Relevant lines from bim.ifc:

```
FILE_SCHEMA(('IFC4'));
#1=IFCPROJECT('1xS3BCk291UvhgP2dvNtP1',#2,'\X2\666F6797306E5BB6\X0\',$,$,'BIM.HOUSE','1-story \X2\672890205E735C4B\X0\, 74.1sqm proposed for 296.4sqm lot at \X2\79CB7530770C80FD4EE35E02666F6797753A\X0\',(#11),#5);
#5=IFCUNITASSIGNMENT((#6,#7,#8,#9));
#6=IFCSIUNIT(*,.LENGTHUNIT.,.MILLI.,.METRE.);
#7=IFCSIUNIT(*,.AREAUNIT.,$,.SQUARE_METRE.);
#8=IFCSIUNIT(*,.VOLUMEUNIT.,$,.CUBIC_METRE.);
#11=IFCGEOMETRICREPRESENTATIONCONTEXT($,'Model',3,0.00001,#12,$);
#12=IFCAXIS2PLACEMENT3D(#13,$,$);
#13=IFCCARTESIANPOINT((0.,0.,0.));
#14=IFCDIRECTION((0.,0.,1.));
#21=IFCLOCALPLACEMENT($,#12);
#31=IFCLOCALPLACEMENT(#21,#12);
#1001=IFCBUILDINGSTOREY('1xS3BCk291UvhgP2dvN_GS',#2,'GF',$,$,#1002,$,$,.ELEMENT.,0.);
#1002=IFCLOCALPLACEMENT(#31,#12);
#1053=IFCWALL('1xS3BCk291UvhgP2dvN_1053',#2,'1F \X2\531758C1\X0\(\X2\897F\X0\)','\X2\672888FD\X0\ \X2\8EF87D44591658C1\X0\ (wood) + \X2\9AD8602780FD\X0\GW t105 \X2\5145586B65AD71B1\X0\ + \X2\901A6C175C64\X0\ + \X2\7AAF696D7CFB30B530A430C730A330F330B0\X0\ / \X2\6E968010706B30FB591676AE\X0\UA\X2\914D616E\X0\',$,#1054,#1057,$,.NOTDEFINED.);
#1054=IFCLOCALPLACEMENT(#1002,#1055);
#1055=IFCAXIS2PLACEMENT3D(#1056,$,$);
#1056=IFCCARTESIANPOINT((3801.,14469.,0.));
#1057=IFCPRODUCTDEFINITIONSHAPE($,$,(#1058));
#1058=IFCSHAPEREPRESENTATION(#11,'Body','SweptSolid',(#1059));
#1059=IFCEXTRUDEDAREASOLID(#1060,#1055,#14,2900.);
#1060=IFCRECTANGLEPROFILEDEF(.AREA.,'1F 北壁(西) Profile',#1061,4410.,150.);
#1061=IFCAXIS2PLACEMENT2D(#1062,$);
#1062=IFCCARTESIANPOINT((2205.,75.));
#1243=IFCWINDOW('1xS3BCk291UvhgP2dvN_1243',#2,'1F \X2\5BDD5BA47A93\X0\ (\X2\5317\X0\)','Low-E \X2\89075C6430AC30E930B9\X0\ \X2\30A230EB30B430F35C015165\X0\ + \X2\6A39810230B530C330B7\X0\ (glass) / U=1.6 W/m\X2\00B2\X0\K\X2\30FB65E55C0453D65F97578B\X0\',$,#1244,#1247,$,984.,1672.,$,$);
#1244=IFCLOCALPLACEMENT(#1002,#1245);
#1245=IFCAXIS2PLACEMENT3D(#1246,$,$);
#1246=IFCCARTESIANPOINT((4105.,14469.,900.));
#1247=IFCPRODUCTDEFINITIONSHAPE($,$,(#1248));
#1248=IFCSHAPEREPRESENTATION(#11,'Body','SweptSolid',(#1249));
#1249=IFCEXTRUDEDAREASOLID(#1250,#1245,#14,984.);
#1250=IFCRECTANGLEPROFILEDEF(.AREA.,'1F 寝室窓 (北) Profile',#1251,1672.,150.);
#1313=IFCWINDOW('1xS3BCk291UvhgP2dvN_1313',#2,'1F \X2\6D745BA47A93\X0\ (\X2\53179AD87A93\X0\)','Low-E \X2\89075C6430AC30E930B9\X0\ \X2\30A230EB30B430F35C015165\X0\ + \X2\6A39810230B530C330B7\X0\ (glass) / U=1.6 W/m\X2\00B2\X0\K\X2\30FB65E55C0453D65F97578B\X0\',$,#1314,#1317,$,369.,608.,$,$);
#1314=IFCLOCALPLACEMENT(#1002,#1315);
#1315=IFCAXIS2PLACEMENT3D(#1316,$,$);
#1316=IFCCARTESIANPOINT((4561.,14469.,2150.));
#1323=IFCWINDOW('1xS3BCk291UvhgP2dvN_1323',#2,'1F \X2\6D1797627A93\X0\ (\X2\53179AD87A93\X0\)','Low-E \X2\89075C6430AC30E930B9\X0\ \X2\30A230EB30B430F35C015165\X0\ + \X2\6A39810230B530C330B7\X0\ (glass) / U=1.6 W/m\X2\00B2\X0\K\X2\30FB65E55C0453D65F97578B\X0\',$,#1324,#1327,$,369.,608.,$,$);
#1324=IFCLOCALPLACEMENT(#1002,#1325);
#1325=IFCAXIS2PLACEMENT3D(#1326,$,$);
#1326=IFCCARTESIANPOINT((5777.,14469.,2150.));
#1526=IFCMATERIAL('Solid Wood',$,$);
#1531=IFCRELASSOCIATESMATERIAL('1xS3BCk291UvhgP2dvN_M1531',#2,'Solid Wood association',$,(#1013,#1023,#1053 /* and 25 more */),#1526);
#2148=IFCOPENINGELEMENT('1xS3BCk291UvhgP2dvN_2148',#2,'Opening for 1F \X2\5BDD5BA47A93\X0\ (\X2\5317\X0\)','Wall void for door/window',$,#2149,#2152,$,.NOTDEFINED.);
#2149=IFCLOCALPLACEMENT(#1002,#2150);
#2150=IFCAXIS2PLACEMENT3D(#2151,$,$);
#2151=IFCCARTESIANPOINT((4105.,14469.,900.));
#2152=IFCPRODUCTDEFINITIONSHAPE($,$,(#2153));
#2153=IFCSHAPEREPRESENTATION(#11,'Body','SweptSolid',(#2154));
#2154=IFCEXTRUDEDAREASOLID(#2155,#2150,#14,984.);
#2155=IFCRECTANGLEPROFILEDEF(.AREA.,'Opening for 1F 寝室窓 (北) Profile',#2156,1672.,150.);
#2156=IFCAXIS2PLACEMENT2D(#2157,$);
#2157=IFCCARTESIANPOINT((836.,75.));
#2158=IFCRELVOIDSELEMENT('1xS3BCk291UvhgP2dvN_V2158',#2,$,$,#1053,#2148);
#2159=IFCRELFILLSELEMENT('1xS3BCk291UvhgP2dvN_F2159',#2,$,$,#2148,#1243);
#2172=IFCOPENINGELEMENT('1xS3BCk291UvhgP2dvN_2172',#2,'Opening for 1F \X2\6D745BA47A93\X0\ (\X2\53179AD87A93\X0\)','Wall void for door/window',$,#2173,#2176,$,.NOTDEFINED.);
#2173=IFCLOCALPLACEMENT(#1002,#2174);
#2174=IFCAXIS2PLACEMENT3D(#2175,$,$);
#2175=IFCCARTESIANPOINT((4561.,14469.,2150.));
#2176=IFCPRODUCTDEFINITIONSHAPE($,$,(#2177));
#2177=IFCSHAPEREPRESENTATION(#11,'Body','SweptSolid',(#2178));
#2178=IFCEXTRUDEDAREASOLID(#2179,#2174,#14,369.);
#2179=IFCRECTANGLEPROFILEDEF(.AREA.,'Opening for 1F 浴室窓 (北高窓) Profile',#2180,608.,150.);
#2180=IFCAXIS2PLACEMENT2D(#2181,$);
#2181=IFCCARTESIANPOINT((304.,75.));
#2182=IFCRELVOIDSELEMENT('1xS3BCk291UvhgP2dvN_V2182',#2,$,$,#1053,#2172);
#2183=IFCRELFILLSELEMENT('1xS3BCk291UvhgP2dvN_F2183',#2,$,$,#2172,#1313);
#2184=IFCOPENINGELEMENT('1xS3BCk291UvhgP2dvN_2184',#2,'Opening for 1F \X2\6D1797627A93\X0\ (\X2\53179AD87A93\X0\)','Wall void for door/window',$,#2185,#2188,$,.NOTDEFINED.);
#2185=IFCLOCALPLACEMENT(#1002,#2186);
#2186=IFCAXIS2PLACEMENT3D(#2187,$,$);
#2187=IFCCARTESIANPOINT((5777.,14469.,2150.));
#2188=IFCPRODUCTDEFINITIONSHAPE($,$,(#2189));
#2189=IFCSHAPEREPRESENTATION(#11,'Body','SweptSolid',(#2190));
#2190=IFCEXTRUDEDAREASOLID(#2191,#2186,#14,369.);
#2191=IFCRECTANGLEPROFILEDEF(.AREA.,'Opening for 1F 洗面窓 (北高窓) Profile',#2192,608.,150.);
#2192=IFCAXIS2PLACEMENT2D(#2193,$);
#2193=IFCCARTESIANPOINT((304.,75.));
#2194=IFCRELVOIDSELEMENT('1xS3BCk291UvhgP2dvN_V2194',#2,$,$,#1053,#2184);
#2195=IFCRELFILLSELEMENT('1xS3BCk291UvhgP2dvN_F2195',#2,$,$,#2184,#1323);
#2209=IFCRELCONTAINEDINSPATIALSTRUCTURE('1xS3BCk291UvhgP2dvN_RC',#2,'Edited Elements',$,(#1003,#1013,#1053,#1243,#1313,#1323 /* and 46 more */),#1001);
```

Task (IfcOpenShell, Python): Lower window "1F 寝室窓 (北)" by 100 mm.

```python
import numpy as np
import ifcopenshell
import ifcopenshell.api.geometry
import ifcopenshell.util.placement
import ifcopenshell.util.unit

model = ifcopenshell.open("bim.ifc")
unit_scale = ifcopenshell.util.unit.calculate_unit_scale(model)

window = model.by_guid("1xS3BCk291UvhgP2dvN_1243")
opening = window.FillsVoids[0].RelatingOpeningElement
dz = -100.0

shift = np.array([0.0, 0.0, dz])
# The window is not placed relative to its opening, so move both.
for product in (opening, window):
    matrix = ifcopenshell.util.placement.get_local_placement(product.ObjectPlacement)
    matrix[:3, 3] += shift
    ifcopenshell.api.geometry.edit_object_placement(model, product=product, matrix=matrix, is_si=False)

print(f"moved by {dz * unit_scale:+.3f} m")

model.write("bim_updated.ifc")
```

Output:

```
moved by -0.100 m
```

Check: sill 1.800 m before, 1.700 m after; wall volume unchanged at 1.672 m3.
